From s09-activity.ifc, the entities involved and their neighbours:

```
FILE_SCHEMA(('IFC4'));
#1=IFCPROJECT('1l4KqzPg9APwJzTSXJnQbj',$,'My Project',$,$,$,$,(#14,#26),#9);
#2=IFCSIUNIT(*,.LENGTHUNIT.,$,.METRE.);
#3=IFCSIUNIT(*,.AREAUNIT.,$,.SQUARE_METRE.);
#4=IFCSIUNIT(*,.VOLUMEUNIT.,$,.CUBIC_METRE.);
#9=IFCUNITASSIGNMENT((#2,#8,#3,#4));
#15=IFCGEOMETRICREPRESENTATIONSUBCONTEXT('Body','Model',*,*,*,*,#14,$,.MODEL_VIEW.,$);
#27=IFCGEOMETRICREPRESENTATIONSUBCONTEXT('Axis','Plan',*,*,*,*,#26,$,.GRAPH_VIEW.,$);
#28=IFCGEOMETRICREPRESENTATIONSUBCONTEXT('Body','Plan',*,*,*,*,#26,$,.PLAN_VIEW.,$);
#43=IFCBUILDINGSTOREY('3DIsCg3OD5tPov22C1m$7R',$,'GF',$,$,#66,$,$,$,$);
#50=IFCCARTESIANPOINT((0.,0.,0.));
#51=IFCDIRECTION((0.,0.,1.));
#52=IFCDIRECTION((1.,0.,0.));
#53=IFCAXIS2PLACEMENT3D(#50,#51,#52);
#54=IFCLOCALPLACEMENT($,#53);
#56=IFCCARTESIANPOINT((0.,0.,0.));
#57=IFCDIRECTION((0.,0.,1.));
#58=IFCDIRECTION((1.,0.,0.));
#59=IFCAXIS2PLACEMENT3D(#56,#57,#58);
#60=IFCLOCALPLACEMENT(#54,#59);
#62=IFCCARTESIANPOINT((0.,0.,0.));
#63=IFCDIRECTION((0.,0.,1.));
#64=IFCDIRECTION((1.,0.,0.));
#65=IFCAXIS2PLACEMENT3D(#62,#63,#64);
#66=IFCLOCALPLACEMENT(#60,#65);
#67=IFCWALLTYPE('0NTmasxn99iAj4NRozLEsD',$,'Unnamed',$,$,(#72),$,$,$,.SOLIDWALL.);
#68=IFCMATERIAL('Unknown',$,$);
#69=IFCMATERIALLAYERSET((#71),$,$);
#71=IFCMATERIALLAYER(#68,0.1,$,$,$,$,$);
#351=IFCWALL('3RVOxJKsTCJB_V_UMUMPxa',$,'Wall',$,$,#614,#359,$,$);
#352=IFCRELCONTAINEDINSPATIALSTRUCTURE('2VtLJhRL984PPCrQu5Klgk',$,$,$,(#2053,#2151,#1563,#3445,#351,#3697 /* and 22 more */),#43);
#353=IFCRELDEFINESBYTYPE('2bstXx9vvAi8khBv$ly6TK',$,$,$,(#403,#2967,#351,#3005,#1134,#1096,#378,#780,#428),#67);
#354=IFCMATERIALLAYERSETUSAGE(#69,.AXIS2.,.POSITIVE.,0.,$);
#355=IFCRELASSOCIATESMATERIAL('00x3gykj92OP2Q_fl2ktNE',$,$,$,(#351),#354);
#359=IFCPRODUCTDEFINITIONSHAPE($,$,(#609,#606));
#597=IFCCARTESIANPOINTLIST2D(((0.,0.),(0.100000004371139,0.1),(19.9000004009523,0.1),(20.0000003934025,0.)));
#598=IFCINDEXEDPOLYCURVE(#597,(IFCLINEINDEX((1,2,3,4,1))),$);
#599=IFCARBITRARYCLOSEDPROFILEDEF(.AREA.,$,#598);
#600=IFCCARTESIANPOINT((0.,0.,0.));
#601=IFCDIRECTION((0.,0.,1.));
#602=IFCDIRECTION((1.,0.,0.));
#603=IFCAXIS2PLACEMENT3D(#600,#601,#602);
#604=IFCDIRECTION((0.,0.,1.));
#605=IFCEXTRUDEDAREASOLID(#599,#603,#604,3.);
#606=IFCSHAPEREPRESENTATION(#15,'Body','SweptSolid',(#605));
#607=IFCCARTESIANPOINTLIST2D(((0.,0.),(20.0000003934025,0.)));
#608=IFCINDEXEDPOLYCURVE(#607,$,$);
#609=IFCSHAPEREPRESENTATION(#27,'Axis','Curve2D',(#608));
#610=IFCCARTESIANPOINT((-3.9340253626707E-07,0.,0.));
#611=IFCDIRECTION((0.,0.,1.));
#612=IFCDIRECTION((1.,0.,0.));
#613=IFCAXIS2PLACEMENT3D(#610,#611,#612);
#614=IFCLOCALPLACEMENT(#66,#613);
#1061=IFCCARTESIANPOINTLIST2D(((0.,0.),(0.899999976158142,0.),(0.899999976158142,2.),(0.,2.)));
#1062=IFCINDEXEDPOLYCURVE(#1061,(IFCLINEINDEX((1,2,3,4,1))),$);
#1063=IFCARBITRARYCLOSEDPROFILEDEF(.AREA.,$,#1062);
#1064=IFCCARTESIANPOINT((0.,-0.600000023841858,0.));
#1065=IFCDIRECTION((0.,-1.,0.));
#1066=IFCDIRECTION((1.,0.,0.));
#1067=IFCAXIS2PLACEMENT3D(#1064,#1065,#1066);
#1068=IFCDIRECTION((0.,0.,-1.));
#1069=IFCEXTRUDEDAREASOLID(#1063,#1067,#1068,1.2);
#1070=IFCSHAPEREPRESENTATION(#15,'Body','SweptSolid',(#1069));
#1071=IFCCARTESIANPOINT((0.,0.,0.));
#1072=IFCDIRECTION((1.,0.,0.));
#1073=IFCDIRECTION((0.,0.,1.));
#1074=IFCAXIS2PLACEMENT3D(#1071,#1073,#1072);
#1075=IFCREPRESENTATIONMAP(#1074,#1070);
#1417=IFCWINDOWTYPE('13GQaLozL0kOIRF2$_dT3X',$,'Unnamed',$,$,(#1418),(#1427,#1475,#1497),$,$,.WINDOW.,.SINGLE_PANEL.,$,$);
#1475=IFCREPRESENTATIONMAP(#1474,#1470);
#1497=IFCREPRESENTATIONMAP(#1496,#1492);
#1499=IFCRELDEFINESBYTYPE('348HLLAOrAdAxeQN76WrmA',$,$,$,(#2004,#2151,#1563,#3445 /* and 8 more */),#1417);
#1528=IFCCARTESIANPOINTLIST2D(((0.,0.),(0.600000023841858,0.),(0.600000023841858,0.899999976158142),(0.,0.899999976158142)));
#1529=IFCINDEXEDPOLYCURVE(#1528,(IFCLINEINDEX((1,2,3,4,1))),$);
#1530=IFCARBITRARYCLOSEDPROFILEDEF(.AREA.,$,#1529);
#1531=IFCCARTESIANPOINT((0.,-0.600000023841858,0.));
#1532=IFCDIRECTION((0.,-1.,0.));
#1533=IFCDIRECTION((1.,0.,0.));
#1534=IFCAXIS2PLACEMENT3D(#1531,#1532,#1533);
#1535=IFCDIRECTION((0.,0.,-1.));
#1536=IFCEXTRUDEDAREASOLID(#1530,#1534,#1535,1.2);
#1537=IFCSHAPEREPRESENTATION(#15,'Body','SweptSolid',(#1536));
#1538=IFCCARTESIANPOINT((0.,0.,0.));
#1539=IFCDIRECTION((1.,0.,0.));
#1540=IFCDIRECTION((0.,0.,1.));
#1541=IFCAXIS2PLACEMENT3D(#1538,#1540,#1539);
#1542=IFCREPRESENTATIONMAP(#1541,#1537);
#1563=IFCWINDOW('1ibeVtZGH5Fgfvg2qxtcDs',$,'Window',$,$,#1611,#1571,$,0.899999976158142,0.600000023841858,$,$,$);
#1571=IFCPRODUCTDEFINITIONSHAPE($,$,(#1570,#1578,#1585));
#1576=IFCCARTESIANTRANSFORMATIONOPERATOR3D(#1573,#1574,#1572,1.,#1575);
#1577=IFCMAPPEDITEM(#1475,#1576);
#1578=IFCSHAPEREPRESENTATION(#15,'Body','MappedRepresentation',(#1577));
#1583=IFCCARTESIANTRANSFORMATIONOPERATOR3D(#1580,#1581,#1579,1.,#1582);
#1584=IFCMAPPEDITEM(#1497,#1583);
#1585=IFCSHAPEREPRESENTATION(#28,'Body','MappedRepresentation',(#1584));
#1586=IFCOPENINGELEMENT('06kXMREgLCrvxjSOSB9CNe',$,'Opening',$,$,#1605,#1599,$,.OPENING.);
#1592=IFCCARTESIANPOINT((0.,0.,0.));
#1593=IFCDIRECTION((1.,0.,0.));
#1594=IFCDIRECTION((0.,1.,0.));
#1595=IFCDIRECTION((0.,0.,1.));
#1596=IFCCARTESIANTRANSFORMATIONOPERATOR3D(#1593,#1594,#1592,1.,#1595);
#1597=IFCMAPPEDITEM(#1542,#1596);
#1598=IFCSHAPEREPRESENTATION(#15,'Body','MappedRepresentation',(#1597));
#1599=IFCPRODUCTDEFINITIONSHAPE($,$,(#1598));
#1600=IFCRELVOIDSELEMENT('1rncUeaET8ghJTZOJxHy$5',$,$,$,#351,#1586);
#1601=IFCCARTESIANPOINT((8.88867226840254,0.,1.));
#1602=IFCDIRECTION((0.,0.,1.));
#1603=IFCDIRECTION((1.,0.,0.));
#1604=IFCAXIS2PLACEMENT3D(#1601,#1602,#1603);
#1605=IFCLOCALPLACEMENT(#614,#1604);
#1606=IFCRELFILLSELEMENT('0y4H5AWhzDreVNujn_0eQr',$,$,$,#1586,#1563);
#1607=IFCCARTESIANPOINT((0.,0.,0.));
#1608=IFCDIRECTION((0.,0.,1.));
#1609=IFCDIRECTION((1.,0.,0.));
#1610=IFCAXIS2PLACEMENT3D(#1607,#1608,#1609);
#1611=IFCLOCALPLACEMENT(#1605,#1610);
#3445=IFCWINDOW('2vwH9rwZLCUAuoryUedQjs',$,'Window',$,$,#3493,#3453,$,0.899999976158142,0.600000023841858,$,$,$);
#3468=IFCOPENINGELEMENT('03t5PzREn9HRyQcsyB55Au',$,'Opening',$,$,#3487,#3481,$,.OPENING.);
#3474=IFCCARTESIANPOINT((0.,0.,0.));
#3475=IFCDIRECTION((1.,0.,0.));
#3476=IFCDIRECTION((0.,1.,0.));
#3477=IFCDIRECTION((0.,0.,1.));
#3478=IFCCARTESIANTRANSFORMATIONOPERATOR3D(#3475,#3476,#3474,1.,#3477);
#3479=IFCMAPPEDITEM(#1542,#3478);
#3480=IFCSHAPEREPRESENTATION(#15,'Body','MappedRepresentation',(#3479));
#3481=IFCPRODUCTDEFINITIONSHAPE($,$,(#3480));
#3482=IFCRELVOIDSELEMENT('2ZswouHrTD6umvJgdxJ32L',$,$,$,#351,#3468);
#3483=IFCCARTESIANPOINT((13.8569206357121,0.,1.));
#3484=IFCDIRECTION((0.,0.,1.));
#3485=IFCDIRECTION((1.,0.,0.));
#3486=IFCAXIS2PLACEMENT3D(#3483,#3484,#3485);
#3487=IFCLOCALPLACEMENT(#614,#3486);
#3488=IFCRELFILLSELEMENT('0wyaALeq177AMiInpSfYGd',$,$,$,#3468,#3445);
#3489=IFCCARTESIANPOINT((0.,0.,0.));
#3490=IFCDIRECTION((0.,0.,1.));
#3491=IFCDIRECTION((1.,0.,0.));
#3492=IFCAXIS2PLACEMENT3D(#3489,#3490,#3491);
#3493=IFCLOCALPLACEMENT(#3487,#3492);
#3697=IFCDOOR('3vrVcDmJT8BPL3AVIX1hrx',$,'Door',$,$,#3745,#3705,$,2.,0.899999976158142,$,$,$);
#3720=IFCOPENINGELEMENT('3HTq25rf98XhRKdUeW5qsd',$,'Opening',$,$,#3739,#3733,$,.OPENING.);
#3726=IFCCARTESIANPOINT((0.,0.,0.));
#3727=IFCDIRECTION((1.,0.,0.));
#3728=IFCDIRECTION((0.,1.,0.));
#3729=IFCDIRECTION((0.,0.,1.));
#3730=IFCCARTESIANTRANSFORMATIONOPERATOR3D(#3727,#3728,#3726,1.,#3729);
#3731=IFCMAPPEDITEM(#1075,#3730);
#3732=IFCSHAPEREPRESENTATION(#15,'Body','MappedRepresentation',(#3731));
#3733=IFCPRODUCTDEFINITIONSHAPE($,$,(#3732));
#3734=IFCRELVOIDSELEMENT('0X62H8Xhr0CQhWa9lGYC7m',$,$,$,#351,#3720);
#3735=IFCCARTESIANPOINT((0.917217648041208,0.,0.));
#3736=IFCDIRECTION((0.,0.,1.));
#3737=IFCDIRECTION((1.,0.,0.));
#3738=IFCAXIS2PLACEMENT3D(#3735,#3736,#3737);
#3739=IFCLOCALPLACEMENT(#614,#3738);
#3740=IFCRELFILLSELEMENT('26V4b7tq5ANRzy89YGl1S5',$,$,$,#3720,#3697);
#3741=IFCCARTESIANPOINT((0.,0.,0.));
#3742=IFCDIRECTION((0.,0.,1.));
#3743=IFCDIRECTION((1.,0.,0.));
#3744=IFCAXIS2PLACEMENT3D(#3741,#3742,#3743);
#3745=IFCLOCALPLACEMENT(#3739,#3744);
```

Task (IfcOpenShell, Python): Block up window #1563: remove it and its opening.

```python
import ifcopenshell
import ifcopenshell.api.feature
import ifcopenshell.api.root
import ifcopenshell.geom
import ifcopenshell.util.shape

model = ifcopenshell.open("s09-activity.ifc")
settings = ifcopenshell.geom.settings()


def volume(element):
    """Net volume in cubic metres, openings subtracted."""
    shape = ifcopenshell.geom.create_shape(settings, element)
    return ifcopenshell.util.shape.get_volume(shape.geometry)


window = model.by_guid("1ibeVtZGH5Fgfvg2qxtcDs")
opening = window.FillsVoids[0].RelatingOpeningElement
wall = opening.VoidsElements[0].RelatingBuildingElement
before = volume(wall)

ifcopenshell.api.root.remove_product(model, product=window)
ifcopenshell.api.feature.remove_feature(model, feature=opening)

after = volume(wall)

print(f"wall volume {before:.3f} -> {after:.3f} m3")

model.write("s09-activity-out.ifc")
```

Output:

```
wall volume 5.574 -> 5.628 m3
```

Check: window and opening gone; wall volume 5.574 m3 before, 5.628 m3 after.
